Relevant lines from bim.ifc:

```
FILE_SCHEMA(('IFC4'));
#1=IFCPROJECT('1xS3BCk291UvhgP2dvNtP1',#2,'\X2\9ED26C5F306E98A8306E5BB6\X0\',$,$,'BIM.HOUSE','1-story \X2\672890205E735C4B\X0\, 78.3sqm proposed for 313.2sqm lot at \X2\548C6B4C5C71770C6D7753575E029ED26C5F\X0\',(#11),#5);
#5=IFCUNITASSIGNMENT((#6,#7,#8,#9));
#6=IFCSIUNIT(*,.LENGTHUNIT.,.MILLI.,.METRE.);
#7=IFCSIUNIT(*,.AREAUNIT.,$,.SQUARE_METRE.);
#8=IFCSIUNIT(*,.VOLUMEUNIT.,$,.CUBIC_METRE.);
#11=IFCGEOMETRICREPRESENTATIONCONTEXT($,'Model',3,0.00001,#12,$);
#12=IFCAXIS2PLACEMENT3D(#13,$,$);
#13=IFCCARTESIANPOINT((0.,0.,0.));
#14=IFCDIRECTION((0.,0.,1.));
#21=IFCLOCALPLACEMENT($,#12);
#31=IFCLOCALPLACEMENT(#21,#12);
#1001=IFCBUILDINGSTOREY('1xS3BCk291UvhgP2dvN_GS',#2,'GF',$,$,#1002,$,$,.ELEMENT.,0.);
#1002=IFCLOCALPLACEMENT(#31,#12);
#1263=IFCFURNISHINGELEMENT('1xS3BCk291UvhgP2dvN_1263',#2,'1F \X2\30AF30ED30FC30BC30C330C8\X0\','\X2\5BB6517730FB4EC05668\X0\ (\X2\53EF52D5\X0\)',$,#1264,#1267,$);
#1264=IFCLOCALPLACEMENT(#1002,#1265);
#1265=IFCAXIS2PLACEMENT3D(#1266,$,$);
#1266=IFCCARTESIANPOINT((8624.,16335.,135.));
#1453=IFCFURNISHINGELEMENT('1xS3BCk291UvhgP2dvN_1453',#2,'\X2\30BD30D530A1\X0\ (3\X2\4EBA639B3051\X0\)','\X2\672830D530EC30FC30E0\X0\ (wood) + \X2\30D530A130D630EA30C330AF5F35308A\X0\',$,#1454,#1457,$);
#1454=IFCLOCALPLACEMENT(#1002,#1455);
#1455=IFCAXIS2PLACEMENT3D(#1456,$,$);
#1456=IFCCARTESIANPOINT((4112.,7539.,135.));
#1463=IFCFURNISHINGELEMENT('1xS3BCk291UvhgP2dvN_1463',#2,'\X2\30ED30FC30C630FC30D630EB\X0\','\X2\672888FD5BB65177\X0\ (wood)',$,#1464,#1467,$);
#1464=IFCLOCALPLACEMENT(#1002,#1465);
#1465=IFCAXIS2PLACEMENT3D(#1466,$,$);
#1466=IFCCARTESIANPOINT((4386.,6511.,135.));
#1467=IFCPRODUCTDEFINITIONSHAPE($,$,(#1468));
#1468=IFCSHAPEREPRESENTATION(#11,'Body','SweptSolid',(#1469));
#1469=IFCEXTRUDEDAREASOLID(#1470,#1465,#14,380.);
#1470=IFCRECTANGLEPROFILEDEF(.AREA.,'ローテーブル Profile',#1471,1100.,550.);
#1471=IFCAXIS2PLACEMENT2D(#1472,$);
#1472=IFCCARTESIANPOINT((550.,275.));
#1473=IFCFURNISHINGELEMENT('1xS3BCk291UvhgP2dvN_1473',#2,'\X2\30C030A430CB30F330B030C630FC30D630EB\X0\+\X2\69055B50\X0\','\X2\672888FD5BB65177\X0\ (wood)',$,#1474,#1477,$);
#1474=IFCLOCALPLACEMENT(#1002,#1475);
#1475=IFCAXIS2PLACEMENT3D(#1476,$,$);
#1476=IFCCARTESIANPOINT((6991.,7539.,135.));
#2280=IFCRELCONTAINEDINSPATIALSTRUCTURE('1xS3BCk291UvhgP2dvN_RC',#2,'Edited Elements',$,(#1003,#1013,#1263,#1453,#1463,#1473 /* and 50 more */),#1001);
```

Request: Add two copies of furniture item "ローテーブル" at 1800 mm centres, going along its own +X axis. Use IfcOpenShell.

```python
import ifcopenshell
import ifcopenshell.api.geometry
import ifcopenshell.api.root
import ifcopenshell.util.element
import ifcopenshell.util.placement
import ifcopenshell.util.unit

model = ifcopenshell.open("bim.ifc")
unit_scale = ifcopenshell.util.unit.calculate_unit_scale(model)


def reuse_history(source, copy):
    """copy_class also copies each property set's owner history, people and application; keep the originals."""
    for rel in copy.IsDefinedBy:
        if rel.is_a("IfcRelDefinesByProperties") and (history := rel.RelatingPropertyDefinition.OwnerHistory):
            rel.RelatingPropertyDefinition.OwnerHistory = source.OwnerHistory
            ifcopenshell.util.element.remove_deep2(model, history)


source = model.by_id(1463)
base = ifcopenshell.util.placement.get_local_placement(source.ObjectPlacement)
step = base[:3, 0] * 1.8 / unit_scale

for i in range(1, 3):
    copy = ifcopenshell.api.root.copy_class(model, product=source)
    copy.Representation = ifcopenshell.util.element.copy_deep(
        model, source.Representation, exclude=["IfcGeometricRepresentationContext", "IfcRepresentationMap"]
    )
    reuse_history(source, copy)
    matrix = base.copy()
    matrix[:3, 3] += i * step
    print("added at", matrix[:3, 3].round(3) + 0.0)
    ifcopenshell.api.geometry.edit_object_placement(model, product=copy, matrix=matrix, is_si=False)

model.write("bim-out.ifc")
```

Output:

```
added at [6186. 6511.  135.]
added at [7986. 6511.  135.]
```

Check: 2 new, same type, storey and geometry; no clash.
